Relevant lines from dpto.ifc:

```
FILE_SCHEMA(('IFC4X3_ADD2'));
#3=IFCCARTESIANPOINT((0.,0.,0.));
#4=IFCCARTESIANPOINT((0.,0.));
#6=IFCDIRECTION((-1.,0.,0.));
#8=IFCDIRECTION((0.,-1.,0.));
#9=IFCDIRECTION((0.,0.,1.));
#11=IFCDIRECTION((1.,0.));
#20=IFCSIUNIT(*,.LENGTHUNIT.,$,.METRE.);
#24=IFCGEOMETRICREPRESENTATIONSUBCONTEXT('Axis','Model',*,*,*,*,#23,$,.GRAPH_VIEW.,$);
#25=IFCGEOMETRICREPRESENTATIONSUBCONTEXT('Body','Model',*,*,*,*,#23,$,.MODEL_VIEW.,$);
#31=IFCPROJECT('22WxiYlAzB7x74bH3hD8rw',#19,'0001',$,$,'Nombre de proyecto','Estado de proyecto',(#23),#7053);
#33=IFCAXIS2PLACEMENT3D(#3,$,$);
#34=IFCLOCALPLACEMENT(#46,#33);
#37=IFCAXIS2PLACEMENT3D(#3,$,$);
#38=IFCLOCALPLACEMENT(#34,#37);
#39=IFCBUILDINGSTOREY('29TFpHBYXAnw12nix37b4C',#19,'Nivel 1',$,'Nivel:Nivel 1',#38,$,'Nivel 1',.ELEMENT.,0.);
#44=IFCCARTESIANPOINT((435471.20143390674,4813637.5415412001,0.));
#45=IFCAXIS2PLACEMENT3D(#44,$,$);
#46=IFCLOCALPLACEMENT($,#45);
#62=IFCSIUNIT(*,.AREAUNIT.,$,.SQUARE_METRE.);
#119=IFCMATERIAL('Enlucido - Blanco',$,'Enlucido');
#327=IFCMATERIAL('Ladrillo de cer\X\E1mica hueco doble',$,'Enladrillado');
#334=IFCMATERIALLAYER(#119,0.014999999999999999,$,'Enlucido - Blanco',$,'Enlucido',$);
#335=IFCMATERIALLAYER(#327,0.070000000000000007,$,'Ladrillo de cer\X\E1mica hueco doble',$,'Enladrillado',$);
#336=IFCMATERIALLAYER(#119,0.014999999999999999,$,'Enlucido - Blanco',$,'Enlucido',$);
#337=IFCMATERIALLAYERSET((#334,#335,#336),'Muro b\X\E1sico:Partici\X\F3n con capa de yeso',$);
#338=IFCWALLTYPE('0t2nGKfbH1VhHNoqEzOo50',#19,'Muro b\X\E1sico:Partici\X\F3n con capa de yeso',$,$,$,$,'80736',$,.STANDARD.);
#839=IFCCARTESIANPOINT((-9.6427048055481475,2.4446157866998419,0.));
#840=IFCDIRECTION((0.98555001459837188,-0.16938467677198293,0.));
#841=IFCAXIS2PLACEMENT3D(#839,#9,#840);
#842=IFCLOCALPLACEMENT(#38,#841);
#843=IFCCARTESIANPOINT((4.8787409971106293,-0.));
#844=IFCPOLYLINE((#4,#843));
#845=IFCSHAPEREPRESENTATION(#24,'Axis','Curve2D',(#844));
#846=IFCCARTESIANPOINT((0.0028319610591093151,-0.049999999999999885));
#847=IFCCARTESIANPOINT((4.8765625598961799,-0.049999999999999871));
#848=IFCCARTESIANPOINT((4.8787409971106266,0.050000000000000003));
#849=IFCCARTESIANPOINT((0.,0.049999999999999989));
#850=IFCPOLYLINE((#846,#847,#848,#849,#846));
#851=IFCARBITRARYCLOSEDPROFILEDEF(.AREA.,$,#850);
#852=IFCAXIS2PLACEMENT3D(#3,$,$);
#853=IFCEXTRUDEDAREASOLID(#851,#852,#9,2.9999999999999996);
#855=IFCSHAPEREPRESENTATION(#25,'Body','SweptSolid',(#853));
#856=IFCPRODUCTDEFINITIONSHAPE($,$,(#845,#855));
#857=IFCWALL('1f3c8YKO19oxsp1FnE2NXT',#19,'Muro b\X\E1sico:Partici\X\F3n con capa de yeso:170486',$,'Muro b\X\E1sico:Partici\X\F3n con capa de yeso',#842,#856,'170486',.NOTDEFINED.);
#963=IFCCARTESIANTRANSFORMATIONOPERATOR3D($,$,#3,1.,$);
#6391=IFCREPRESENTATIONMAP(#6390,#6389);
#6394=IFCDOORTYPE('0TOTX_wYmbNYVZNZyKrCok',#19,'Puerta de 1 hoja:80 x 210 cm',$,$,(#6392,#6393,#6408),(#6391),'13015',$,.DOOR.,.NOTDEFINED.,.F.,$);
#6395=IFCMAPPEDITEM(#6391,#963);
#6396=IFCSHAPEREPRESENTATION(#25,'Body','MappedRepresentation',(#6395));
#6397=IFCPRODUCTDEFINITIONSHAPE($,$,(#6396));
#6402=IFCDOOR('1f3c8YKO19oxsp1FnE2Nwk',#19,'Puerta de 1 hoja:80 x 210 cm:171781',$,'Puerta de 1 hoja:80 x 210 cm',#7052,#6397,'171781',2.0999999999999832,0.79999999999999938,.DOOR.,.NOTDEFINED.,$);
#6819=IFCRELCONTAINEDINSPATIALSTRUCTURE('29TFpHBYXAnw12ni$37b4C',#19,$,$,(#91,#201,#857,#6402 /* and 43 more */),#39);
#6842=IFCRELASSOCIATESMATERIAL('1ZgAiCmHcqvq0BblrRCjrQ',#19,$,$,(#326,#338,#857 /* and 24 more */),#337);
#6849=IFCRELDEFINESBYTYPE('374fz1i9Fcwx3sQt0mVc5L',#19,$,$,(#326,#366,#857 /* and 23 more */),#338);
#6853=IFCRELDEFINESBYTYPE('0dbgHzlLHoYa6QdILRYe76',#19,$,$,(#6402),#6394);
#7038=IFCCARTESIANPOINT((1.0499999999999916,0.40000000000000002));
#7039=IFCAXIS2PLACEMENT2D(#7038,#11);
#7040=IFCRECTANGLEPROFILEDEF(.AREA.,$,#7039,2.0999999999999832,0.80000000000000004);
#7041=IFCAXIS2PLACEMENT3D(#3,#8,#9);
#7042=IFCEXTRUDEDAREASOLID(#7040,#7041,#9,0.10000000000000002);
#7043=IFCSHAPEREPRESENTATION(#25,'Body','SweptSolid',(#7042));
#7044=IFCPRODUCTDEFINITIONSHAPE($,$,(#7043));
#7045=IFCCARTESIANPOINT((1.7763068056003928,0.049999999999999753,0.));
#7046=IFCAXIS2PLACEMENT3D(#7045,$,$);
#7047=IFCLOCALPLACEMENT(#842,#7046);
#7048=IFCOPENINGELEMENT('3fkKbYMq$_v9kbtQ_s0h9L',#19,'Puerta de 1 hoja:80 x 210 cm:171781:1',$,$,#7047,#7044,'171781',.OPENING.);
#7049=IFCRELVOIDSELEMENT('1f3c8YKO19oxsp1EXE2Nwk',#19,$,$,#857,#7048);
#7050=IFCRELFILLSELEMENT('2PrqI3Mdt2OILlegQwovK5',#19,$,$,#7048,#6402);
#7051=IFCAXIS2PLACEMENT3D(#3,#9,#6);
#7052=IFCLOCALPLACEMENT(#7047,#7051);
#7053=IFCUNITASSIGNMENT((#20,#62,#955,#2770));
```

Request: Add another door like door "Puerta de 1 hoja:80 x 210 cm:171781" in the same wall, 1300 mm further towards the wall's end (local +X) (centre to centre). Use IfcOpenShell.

```python
import ifcopenshell
import ifcopenshell.api.feature
import ifcopenshell.api.geometry
import ifcopenshell.api.root
import ifcopenshell.geom
import ifcopenshell.util.element
import ifcopenshell.util.placement
import ifcopenshell.util.shape
import ifcopenshell.util.unit

model = ifcopenshell.open("dpto.ifc")
unit_scale = ifcopenshell.util.unit.calculate_unit_scale(model)
settings = ifcopenshell.geom.settings()


def volume(element):
    """Net volume in cubic metres, openings subtracted."""
    shape = ifcopenshell.geom.create_shape(settings, element)
    return ifcopenshell.util.shape.get_volume(shape.geometry)


def reuse_history(source, copy):
    """copy_class also copies each property set's owner history, people and application; keep the originals."""
    for rel in copy.IsDefinedBy:
        if rel.is_a("IfcRelDefinesByProperties") and (history := rel.RelatingPropertyDefinition.OwnerHistory):
            rel.RelatingPropertyDefinition.OwnerHistory = source.OwnerHistory
            ifcopenshell.util.element.remove_deep2(model, history)


door = model.by_guid("1f3c8YKO19oxsp1FnE2Nwk")
opening = door.FillsVoids[0].RelatingOpeningElement
wall = opening.VoidsElements[0].RelatingBuildingElement
before = volume(wall)
shift = ifcopenshell.util.placement.get_local_placement(wall.ObjectPlacement)[:3, 0] * 1.3 / unit_scale

# copy_class copies the void relationship, type, container and properties, but no geometry.
new_opening = ifcopenshell.api.root.copy_class(model, product=opening)
new_opening.Representation = ifcopenshell.util.element.copy_deep(
    model, opening.Representation, exclude=["IfcGeometricRepresentationContext", "IfcRepresentationMap"]
)
new_opening.Name = "Puerta de 1 hoja:80 x 210 cm"
new_opening.Tag = None
new_door = ifcopenshell.api.root.copy_class(model, product=door)
new_door.Representation = ifcopenshell.util.element.copy_deep(
    model, door.Representation, exclude=["IfcGeometricRepresentationContext", "IfcRepresentationMap"]
)
new_door.Name = "Puerta de 1 hoja:80 x 210 cm"
new_door.Tag = None
reuse_history(door, new_door)
ifcopenshell.api.feature.add_filling(model, opening=new_opening, element=new_door)

for old, new in ((opening, new_opening), (door, new_door)):
    matrix = ifcopenshell.util.placement.get_local_placement(old.ObjectPlacement)
    matrix[:3, 3] += shift
    ifcopenshell.api.geometry.edit_object_placement(model, product=new, matrix=matrix, is_si=False)

after = volume(wall)

print(f"wall volume {before:.3f} -> {after:.3f} m3")

model.write("dpto_v2.ifc")
```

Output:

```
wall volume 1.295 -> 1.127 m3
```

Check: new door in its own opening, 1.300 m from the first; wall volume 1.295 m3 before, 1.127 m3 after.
